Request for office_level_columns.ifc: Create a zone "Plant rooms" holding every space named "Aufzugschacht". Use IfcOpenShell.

First a look at what the model holds.

```python
import ifcopenshell

model = ifcopenshell.open("office_level_columns.ifc")
print(model.schema)
seen = {}
for space in model.by_type("IfcSpace"):
    seen[space.LongName] = seen.get(space.LongName, 0) + 1
for name, count in sorted(seen.items(), key=str):
    print(count, "x", name)
print("zones:", [z.Name for z in model.by_type("IfcZone")][:20])
```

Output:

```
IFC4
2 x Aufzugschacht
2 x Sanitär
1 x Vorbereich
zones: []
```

```python
import ifcopenshell
import ifcopenshell.api.group
import ifcopenshell.api.root

model = ifcopenshell.open("office_level_columns.ifc")

names = {"Aufzugschacht"}
spaces = [s for s in model.by_type("IfcSpace") if s.LongName in names]

zone = ifcopenshell.api.root.create_entity(model, ifc_class="IfcZone", name="Plant rooms")
ifcopenshell.api.group.assign_group(model, products=spaces, group=zone)
print(len(spaces), "spaces in", zone.Name)

model.write("office_level_columns_v2.ifc")
```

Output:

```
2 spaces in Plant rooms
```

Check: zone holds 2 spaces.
